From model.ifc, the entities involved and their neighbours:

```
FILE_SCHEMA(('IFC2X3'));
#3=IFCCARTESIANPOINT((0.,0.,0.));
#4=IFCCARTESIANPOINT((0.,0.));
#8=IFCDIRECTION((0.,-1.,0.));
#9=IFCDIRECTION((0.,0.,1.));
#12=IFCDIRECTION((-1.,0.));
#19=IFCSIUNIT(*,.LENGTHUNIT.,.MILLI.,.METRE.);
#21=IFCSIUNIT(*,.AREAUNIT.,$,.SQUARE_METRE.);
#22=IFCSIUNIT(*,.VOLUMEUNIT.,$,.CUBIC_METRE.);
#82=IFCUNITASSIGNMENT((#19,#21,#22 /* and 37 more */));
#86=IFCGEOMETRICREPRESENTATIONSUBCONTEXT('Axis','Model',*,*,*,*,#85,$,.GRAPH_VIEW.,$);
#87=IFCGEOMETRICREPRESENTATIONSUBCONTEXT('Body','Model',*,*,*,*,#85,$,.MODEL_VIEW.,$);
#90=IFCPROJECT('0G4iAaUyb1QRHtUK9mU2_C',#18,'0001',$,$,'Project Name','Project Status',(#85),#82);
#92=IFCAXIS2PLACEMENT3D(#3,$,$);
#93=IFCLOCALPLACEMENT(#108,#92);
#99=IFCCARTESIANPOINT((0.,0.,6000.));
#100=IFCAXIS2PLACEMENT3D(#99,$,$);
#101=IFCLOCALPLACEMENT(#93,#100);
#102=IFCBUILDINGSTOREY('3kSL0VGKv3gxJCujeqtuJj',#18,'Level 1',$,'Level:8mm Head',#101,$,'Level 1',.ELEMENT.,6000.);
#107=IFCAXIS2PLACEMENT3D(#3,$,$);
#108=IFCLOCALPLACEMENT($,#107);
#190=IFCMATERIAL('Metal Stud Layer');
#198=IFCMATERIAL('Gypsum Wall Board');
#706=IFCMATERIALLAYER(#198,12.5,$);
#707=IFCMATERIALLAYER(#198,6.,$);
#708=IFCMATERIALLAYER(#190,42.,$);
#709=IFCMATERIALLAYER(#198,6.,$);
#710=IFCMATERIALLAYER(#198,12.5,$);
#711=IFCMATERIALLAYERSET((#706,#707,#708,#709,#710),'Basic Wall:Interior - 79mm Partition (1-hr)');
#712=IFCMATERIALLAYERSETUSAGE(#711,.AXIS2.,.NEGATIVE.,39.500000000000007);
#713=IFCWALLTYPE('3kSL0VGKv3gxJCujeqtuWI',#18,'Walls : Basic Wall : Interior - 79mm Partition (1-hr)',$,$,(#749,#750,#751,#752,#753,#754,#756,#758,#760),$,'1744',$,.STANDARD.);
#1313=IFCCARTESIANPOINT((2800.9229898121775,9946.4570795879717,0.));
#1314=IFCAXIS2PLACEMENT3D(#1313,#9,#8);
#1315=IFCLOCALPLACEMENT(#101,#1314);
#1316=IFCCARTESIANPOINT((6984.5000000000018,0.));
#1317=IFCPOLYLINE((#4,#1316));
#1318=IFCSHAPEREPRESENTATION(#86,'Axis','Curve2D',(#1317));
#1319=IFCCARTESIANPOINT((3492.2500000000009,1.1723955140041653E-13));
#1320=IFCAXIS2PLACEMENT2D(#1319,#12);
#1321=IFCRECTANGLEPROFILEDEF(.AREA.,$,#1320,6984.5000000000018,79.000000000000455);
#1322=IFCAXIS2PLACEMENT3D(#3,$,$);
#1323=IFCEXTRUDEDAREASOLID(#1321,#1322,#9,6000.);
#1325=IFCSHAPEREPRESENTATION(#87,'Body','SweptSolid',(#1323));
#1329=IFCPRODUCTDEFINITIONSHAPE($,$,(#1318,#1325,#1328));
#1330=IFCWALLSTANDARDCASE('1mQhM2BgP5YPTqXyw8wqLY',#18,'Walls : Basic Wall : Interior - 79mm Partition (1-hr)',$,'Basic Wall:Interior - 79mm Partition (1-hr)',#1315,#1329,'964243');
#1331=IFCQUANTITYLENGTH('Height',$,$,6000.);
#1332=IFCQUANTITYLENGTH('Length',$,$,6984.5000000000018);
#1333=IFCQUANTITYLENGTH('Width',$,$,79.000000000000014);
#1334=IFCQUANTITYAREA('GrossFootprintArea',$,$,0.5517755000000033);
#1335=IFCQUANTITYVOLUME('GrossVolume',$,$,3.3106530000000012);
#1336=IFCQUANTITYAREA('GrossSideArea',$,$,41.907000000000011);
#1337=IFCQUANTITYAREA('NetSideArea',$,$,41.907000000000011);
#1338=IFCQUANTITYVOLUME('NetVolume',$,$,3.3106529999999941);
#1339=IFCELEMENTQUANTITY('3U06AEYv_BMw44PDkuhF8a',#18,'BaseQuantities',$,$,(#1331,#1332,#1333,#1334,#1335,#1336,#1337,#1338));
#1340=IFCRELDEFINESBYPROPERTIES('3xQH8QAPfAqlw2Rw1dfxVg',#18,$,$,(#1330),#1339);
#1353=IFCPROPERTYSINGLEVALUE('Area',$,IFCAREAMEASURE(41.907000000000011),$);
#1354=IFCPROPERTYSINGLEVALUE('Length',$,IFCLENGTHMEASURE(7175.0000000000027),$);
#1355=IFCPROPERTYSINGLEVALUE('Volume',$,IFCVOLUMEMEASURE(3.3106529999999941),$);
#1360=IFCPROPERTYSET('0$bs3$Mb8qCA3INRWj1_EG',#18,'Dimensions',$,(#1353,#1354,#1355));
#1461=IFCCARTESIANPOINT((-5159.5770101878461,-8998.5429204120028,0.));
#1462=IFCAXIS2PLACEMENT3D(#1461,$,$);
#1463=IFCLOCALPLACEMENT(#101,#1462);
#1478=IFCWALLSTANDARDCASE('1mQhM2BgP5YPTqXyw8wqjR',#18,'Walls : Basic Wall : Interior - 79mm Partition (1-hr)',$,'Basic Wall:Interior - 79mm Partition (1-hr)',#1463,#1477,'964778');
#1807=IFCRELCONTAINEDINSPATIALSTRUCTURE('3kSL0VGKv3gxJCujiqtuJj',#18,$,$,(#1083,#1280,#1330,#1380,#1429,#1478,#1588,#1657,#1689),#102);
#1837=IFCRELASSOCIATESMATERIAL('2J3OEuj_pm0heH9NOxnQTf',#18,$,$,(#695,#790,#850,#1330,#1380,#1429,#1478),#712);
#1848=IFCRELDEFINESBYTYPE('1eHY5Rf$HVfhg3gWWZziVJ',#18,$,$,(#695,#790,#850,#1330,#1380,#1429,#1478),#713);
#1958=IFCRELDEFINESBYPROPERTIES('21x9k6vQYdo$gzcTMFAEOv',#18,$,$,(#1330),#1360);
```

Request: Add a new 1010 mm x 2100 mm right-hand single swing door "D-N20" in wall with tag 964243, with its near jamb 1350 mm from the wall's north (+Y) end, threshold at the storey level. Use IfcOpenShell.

```python
import numpy as np
import ifcopenshell
import ifcopenshell.api.feature
import ifcopenshell.api.geometry
import ifcopenshell.api.pset
import ifcopenshell.api.root
import ifcopenshell.api.spatial
import ifcopenshell.api.type
import ifcopenshell.geom
import ifcopenshell.util.element
import ifcopenshell.util.placement
import ifcopenshell.util.representation
import ifcopenshell.util.shape
import ifcopenshell.util.unit

model = ifcopenshell.open("model.ifc")
unit_scale = ifcopenshell.util.unit.calculate_unit_scale(model)
area_scale = ifcopenshell.util.unit.calculate_unit_scale(model, "AREAUNIT")
volume_scale = ifcopenshell.util.unit.calculate_unit_scale(model, "VOLUMEUNIT")
settings = ifcopenshell.geom.settings()


def volume(element):
    """Net volume in cubic metres, openings subtracted."""
    shape = ifcopenshell.geom.create_shape(settings, element)
    return ifcopenshell.util.shape.get_volume(shape.geometry)


wall = model.by_guid("1mQhM2BgP5YPTqXyw8wqLY")
storey = ifcopenshell.util.element.get_container(wall, ifc_class="IfcBuildingStorey")
context = ifcopenshell.util.representation.get_context(model, "Model", "Body", "MODEL_VIEW")
before = volume(wall)

width, height, from_end, sill = 1.01, 2.1, 1.35, 0.0  # metres

# The wall runs along its own X axis, and the end named is its -X end.
wall_shape = ifcopenshell.geom.create_shape(settings, wall)
x, y, z = ifcopenshell.util.shape.get_vertices(wall_shape.geometry).T
start = x.min() + from_end
face, thickness = float(y.min()), float(y.max() - y.min())
wall_matrix = ifcopenshell.util.placement.get_local_placement(wall.ObjectPlacement)
level = ifcopenshell.util.placement.get_local_placement(storey.ObjectPlacement)[2, 3]


def in_wall(x, y):
    """Placement at x, y metres in the wall's axes, at sill height."""
    matrix = wall_matrix.copy()
    matrix[:, 3] = wall_matrix @ np.array([x / unit_scale, y / unit_scale, 0.0, 1.0])
    matrix[2, 3] = level + sill / unit_scale
    return matrix


# Opening: a box that overshoots both wall faces by 50 mm.
opening = ifcopenshell.api.root.create_entity(model, ifc_class="IfcOpeningElement")
box = ifcopenshell.api.geometry.add_wall_representation(
    model, context=context, length=width, height=height, thickness=thickness + 0.1
)
ifcopenshell.api.geometry.assign_representation(model, product=opening, representation=box)
ifcopenshell.api.geometry.edit_object_placement(model, product=opening, matrix=in_wall(start, face - 0.05), is_si=False)
ifcopenshell.api.feature.add_feature(model, feature=opening, element=wall)

door = ifcopenshell.api.root.create_entity(model, ifc_class="IfcDoor", name="D-N20")
door.OverallWidth, door.OverallHeight = width / unit_scale, height / unit_scale
body = ifcopenshell.api.geometry.add_door_representation(
    model,
    context=context,
    overall_width=door.OverallWidth,
    overall_height=door.OverallHeight,
    operation_type="SINGLE_SWING_RIGHT",
    lining_properties={"LiningDepth": thickness / unit_scale, "ThresholdDepth": thickness / unit_scale},
)
ifcopenshell.api.geometry.assign_representation(model, product=door, representation=body)
ifcopenshell.api.spatial.assign_container(model, products=[door], relating_structure=storey)
fills = ifcopenshell.api.feature.add_filling(model, opening=opening, element=door)
fills.OwnerHistory = door.OwnerHistory  # required in IFC2X3

# IFC2X3 keeps the operation on the door style.
style = ifcopenshell.api.root.create_entity(model, ifc_class="IfcDoorStyle", name="D-N20")
style.OperationType, style.ConstructionType = "SINGLE_SWING_RIGHT", "NOTDEFINED"
style.ParameterTakesPrecedence = style.Sizeable = False
ifcopenshell.api.type.assign_type(model, related_objects=[door], relating_type=style)

# The lining spans the wall, so the door starts at the wall face.
ifcopenshell.api.geometry.edit_object_placement(model, product=door, matrix=in_wall(start, face), is_si=False)

after = volume(wall)

# Update the wall's stored quantities.
qto = model.by_id(ifcopenshell.util.element.get_pset(wall, "BaseQuantities", should_inherit=False)["id"])
ifcopenshell.api.pset.edit_qto(model, qto=qto, properties={
    "NetSideArea": after / thickness / area_scale,
    "NetVolume": after / volume_scale,
})
pset = model.by_id(ifcopenshell.util.element.get_pset(wall, "Dimensions", should_inherit=False)["id"])
ifcopenshell.api.pset.edit_pset(model, pset=pset, properties={
    "Area": model.create_entity("IfcAreaMeasure", after / thickness / area_scale),
    "Volume": model.create_entity("IfcVolumeMeasure", after / volume_scale),
})

print(f"wall volume {before:.3f} -> {after:.3f} m3")

model.write("model_edited.ifc")
```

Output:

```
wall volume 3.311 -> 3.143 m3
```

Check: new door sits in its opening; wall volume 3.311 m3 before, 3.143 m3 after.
